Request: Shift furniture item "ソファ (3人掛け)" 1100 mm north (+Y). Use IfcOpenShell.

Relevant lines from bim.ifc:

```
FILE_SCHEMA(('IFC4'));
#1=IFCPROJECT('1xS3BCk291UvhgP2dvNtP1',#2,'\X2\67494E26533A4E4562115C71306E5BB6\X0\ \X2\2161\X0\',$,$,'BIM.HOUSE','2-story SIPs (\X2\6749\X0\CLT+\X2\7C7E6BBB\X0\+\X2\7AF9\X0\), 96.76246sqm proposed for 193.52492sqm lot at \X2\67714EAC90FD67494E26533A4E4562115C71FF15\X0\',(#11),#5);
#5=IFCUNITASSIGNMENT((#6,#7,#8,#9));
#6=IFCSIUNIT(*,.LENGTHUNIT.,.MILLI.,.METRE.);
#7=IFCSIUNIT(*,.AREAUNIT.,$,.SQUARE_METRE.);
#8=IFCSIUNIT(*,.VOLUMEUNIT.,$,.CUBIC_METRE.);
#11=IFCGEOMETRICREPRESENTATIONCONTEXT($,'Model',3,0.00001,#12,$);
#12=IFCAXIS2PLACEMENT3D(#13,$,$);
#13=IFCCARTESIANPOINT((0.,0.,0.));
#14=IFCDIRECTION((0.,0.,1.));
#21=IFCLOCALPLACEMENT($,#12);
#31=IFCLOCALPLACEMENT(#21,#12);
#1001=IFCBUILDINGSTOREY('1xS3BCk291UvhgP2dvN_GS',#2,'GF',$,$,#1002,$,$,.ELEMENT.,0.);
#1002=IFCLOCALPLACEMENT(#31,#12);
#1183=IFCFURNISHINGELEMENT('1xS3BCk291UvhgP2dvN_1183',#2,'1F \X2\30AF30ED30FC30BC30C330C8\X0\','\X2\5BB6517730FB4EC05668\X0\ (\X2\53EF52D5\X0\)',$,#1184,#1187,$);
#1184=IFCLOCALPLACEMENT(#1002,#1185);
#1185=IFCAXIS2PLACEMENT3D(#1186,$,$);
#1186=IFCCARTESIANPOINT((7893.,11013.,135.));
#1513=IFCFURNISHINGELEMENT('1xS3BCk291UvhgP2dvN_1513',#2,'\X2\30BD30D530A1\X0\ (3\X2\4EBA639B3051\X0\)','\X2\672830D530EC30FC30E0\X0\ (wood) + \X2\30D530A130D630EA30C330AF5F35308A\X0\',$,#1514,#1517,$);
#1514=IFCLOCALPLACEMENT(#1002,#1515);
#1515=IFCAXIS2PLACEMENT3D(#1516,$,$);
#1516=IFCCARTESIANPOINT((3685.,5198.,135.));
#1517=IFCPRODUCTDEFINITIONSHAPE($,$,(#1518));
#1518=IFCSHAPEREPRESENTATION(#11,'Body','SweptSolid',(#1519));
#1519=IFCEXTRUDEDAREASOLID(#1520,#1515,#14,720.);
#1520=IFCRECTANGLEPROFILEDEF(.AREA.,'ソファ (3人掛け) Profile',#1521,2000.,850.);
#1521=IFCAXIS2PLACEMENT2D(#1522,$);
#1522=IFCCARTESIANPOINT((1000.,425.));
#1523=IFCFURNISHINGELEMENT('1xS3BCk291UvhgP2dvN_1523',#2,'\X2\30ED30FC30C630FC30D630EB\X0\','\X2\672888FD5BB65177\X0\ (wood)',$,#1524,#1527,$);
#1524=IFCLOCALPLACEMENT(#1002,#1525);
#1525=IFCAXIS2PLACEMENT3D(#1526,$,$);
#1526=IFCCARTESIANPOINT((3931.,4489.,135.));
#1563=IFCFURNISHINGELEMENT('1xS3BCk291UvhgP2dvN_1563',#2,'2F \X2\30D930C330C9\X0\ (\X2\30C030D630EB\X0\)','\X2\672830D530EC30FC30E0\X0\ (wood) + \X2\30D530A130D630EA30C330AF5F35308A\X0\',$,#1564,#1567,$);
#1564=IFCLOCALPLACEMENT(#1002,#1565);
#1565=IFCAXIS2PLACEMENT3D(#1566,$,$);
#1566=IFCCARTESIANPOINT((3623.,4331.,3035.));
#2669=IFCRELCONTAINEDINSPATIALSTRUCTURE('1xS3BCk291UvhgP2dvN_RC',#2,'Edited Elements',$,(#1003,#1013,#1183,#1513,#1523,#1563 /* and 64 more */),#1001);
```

```python
import ifcopenshell
import ifcopenshell.api.geometry
import ifcopenshell.util.placement

model = ifcopenshell.open("bim.ifc")

item = model.by_id(1513)
matrix = ifcopenshell.util.placement.get_local_placement(item.ObjectPlacement)
matrix[1, 3] += 1100.0
ifcopenshell.api.geometry.edit_object_placement(model, product=item, matrix=matrix, is_si=False)

print(ifcopenshell.util.placement.get_local_placement(item.ObjectPlacement).round(3) + 0.0)

model.write("bim_updated.ifc")
```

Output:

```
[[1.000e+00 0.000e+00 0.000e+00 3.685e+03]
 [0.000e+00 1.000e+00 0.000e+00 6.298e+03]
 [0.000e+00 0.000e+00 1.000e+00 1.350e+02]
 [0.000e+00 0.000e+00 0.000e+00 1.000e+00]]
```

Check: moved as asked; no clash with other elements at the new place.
